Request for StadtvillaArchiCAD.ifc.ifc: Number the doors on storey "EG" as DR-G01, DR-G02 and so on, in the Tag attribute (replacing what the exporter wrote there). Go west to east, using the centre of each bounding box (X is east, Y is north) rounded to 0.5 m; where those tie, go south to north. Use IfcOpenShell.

First a look at what the model holds.

```python
import ifcopenshell
import ifcopenshell.util.element
import ifcopenshell.util.placement

model = ifcopenshell.open("StadtvillaArchiCAD.ifc.ifc")
print(model.schema)
storey = next(s for s in model.by_type("IfcBuildingStorey") if s.Name == "EG")
doors = [e for e in ifcopenshell.util.element.get_decomposition(storey) if e.is_a("IfcDoor")]
for e in sorted(doors, key=lambda e: e.id()):
    origin = ifcopenshell.util.placement.get_local_placement(e.ObjectPlacement)[:3, 3]
    print(e.id(), e.Tag, e.Name, origin.round(2) + 0.0, sep=" | ")
```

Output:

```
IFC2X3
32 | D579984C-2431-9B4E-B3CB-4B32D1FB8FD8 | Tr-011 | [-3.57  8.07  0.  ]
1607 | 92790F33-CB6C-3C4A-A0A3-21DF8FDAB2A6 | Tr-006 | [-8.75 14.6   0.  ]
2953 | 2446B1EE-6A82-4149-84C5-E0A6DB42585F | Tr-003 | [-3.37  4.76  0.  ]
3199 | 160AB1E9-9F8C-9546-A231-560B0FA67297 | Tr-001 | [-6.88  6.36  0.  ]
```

```python
import ifcopenshell
import ifcopenshell.geom
import ifcopenshell.util.element
import ifcopenshell.util.shape

model = ifcopenshell.open("StadtvillaArchiCAD.ifc.ifc")
settings = ifcopenshell.geom.settings()
settings.set("use-world-coords", True)


def centre(element):
    shape = ifcopenshell.geom.create_shape(settings, element)
    return ifcopenshell.util.shape.get_bbox_centroid(shape.geometry)


storey = next(s for s in model.by_type("IfcBuildingStorey") if s.Name == "EG")
doors = [e for e in ifcopenshell.util.element.get_decomposition(storey) if e.is_a("IfcDoor")]

# Insertion points can sit at a corner or the storey origin, so sort by the geometry (in metres).
centres = {e: centre(e) for e in doors}
doors.sort(key=lambda e: (round(centres[e][0] / 0.5), centres[e][1]))

for i, e in enumerate(doors, start=1):
    number = f"DR-G{i:02d}"
    e.Tag = number
    print(e.id(), number)

model.write("StadtvillaArchiCAD.ifc-out.ifc")
```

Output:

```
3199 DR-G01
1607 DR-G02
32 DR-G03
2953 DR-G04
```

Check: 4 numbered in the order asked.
